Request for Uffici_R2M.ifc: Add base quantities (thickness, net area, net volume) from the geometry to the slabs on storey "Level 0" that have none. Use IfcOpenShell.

First a look at what the model holds.

```python
import ifcopenshell
import ifcopenshell.util.element
import ifcopenshell.util.unit

model = ifcopenshell.open("Uffici_R2M.ifc")
print(model.schema)
for unit_type in ("LENGTHUNIT", "AREAUNIT", "VOLUMEUNIT"):
    print(unit_type, ifcopenshell.util.unit.calculate_unit_scale(model, unit_type))
storey = next(s for s in model.by_type("IfcBuildingStorey") if s.Name == "Level 0")
slabs = [e for e in ifcopenshell.util.element.get_decomposition(storey) if e.is_a("IfcSlab")]
for e in sorted(slabs, key=lambda e: e.id()):
    print(e.id(), e.is_a(), e.Name, list(ifcopenshell.util.element.get_psets(e, qtos_only=True)), sep=" | ")
```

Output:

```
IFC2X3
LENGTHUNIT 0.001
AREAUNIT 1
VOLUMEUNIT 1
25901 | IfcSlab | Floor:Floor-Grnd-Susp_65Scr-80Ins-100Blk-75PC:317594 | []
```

```python
import ifcopenshell
import ifcopenshell.api.pset
import ifcopenshell.geom
import ifcopenshell.util.element
import ifcopenshell.util.shape
import ifcopenshell.util.unit

model = ifcopenshell.open("Uffici_R2M.ifc")
unit_scale = ifcopenshell.util.unit.calculate_unit_scale(model)
area_scale = ifcopenshell.util.unit.calculate_unit_scale(model, "AREAUNIT")
volume_scale = ifcopenshell.util.unit.calculate_unit_scale(model, "VOLUMEUNIT")
settings = ifcopenshell.geom.settings()

storey = next(s for s in model.by_type("IfcBuildingStorey") if s.Name == "Level 0")
slabs = [e for e in ifcopenshell.util.element.get_decomposition(storey) if e.is_a("IfcSlab")]

for e in sorted(slabs, key=lambda e: e.id()):
    if ifcopenshell.util.element.get_psets(e, qtos_only=True, should_inherit=False):
        continue
    # Geometry comes back in metres, in the element's own axes.
    shape = ifcopenshell.geom.create_shape(settings, e)
    values = {
        "Width": ifcopenshell.util.shape.get_z(shape.geometry) / unit_scale,
        "NetArea": ifcopenshell.util.shape.get_footprint_area(shape.geometry) / area_scale,
        "NetVolume": ifcopenshell.util.shape.get_volume(shape.geometry) / volume_scale,
    }
    qto = ifcopenshell.api.pset.add_qto(model, product=e, name="BaseQuantities")
    ifcopenshell.api.pset.edit_qto(model, qto=qto, properties=values)
    print(e.id(), {k: round(v, 3) for k, v in values.items()})

model.write("Uffici_R2M_updated.ifc")
```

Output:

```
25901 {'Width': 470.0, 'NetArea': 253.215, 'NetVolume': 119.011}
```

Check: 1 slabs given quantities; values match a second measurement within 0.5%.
